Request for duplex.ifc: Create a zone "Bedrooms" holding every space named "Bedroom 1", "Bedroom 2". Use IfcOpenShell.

First a look at what the model holds.

```python
import ifcopenshell

model = ifcopenshell.open("duplex.ifc")
print(model.schema)
seen = {}
for space in model.by_type("IfcSpace"):
    seen[space.LongName] = seen.get(space.LongName, 0) + 1
for name, count in sorted(seen.items(), key=str):
    print(count, "x", name)
print("zones:", [z.Name for z in model.by_type("IfcZone")][:20])
```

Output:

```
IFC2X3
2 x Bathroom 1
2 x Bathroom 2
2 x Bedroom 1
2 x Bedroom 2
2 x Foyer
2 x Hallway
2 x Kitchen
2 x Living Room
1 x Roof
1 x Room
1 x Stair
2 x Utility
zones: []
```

```python
import ifcopenshell
import ifcopenshell.api.group
import ifcopenshell.api.root

model = ifcopenshell.open("duplex.ifc")

names = {"Bedroom 1", "Bedroom 2"}
spaces = [s for s in model.by_type("IfcSpace") if s.LongName in names]

zone = ifcopenshell.api.root.create_entity(model, ifc_class="IfcZone", name="Bedrooms")
ifcopenshell.api.group.assign_group(model, products=spaces, group=zone)
print(len(spaces), "spaces in", zone.Name)

model.write("duplex_edited.ifc")
```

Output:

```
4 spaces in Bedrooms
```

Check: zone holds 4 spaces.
